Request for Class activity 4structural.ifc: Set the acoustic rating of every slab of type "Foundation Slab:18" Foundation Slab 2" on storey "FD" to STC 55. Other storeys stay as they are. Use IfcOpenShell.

First a look at what the model holds.

```python
import ifcopenshell
import ifcopenshell.util.element

model = ifcopenshell.open("Class activity 4structural.ifc")
print(model.schema)
storey = next(s for s in model.by_type("IfcBuildingStorey") if s.Name == "FD")
slabs = [e for e in ifcopenshell.util.element.get_decomposition(storey) if e.is_a("IfcSlab")]
seen = {}
for e in slabs:
    element_type = ifcopenshell.util.element.get_type(e)
    key = (element_type.Name if element_type != e and element_type else None, ifcopenshell.util.element.get_pset(e, "Pset_SlabCommon", "AcousticRating"))
    seen[key] = seen.get(key, 0) + 1
for (name, value), count in sorted(seen.items(), key=str):
    print(count, "x", name, "|", value)
```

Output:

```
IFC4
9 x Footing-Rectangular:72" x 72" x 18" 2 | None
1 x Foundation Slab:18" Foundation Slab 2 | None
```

```python
import ifcopenshell
import ifcopenshell.api.pset
import ifcopenshell.util.element

model = ifcopenshell.open("Class activity 4structural.ifc")

storey = next(s for s in model.by_type("IfcBuildingStorey") if s.Name == "FD")
slabs = [e for e in ifcopenshell.util.element.get_decomposition(storey) if e.is_a("IfcSlab")]

count = 0
for e in slabs:
    element_type = ifcopenshell.util.element.get_type(e)
    if element_type in (None, e) or element_type.Name != 'Foundation Slab:18" Foundation Slab 2':
        continue
    # add_pset returns the element's existing set when there is one.
    pset = ifcopenshell.api.pset.add_pset(model, product=e, name="Pset_SlabCommon")
    ifcopenshell.api.pset.edit_pset(model, pset=pset, properties={"AcousticRating": "STC 55"})
    count += 1

print(count, "slabs updated")

model.write("Class activity 4structural_edited.ifc")
```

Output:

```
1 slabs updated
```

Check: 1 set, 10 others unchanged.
